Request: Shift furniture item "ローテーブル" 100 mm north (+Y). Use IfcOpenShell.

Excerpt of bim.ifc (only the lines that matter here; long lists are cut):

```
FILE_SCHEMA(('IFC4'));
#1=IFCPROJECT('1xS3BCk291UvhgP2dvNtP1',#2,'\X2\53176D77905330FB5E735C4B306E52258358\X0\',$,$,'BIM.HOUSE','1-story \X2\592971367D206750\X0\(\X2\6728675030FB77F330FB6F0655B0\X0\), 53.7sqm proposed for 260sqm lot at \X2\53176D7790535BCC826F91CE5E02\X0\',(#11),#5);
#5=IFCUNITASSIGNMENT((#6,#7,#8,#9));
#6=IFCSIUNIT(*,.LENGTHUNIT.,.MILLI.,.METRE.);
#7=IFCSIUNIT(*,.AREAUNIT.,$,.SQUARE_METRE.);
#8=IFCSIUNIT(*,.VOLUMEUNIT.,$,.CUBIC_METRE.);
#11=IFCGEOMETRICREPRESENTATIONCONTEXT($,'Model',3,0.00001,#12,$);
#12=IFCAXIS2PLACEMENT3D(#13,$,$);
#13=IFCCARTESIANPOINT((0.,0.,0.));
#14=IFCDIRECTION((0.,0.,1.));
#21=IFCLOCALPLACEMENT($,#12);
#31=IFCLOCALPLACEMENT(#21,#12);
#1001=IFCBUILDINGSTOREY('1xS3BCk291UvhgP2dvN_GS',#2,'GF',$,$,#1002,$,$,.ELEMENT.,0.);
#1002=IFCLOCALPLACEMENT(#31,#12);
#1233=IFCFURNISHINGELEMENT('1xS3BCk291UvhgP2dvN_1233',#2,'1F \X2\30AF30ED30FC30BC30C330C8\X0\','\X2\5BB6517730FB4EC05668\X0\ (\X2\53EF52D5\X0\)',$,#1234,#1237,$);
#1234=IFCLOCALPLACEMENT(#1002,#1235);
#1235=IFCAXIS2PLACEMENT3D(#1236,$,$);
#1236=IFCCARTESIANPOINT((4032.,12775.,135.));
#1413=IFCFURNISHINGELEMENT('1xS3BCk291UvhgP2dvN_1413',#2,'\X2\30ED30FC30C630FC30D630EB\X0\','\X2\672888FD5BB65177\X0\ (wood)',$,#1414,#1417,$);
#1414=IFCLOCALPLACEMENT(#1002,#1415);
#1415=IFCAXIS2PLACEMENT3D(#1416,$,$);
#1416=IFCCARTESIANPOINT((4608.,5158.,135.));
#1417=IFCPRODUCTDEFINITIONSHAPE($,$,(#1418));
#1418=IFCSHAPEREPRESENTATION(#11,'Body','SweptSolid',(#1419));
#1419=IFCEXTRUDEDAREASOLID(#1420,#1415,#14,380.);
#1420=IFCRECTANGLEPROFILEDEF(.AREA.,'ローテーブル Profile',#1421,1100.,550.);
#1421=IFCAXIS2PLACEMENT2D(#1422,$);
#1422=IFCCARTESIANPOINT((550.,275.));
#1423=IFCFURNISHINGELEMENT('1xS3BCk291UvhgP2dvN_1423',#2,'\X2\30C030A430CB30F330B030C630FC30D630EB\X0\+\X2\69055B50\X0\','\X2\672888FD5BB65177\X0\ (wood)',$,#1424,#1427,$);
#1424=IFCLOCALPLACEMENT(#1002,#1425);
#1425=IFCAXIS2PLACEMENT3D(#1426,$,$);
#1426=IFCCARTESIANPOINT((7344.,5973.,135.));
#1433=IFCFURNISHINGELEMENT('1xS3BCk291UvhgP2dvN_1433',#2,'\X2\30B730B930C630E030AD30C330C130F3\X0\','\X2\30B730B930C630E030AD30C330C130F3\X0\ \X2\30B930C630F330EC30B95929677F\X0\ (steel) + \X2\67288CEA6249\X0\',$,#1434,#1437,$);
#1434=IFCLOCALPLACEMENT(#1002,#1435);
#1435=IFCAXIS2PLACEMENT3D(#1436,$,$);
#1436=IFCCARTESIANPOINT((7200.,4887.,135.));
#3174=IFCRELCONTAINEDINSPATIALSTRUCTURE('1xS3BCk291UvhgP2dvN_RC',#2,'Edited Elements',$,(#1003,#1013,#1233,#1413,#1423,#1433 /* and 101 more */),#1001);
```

```python
import ifcopenshell
import ifcopenshell.api.geometry
import ifcopenshell.util.placement
import ifcopenshell.util.unit

model = ifcopenshell.open("bim.ifc")
unit_scale = ifcopenshell.util.unit.calculate_unit_scale(model)

item = model.by_id(1413)
matrix = ifcopenshell.util.placement.get_local_placement(item.ObjectPlacement)
matrix[1, 3] += 0.1 / unit_scale
ifcopenshell.api.geometry.edit_object_placement(model, product=item, matrix=matrix, is_si=False)

print(ifcopenshell.util.placement.get_local_placement(item.ObjectPlacement).round(3) + 0.0)

model.write("bim_edited.ifc")
```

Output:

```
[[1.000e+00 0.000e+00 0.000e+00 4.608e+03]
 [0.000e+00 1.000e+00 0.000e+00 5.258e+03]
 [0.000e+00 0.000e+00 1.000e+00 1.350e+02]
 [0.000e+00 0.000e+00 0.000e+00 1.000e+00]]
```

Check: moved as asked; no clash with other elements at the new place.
